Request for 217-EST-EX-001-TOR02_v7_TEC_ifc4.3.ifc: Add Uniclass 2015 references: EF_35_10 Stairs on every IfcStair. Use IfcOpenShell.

First a look at what the model holds.

```python
import ifcopenshell

model = ifcopenshell.open("217-EST-EX-001-TOR02_v7_TEC_ifc4.3.ifc")
print(model.schema)
print("classifications:", [c.Name for c in model.by_type("IfcClassification")])
for ifc_class in ("IfcDoor", "IfcRoof", "IfcStair", "IfcWall", "IfcWindow"):
    print(ifc_class, len(model.by_type(ifc_class)))
```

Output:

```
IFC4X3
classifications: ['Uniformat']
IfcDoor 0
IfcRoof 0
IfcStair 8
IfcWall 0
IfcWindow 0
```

```python
import ifcopenshell
import ifcopenshell.api.classification

model = ifcopenshell.open("217-EST-EX-001-TOR02_v7_TEC_ifc4.3.ifc")

system = ifcopenshell.api.classification.add_classification(model, classification="Uniclass 2015")

codes = {
    "IfcStair": ("EF_35_10", "Stairs"),
}
for ifc_class, (code, name) in codes.items():
    products = model.by_type(ifc_class)
    ifcopenshell.api.classification.add_reference(
        model, products=products, classification=system, identification=code, name=name
    )
    print(code, len(products))

model.write("217-EST-EX-001-TOR02_v7_TEC_ifc4.3_updated.ifc")
```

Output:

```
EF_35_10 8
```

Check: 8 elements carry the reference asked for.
